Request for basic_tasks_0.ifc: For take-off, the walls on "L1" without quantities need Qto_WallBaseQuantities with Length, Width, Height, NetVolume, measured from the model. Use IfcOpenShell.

First a look at what the model holds.

```python
import ifcopenshell
import ifcopenshell.util.element
import ifcopenshell.util.unit

model = ifcopenshell.open("basic_tasks_0.ifc")
print(model.schema)
for unit_type in ("LENGTHUNIT", "AREAUNIT", "VOLUMEUNIT"):
    print(unit_type, ifcopenshell.util.unit.calculate_unit_scale(model, unit_type))
storey = next(s for s in model.by_type("IfcBuildingStorey") if s.Name == "L1")
walls = [e for e in ifcopenshell.util.element.get_decomposition(storey) if e.is_a("IfcWall")]
for e in sorted(walls, key=lambda e: e.id()):
    print(e.id(), e.is_a(), e.Name, list(ifcopenshell.util.element.get_psets(e, qtos_only=True)), sep=" | ")
```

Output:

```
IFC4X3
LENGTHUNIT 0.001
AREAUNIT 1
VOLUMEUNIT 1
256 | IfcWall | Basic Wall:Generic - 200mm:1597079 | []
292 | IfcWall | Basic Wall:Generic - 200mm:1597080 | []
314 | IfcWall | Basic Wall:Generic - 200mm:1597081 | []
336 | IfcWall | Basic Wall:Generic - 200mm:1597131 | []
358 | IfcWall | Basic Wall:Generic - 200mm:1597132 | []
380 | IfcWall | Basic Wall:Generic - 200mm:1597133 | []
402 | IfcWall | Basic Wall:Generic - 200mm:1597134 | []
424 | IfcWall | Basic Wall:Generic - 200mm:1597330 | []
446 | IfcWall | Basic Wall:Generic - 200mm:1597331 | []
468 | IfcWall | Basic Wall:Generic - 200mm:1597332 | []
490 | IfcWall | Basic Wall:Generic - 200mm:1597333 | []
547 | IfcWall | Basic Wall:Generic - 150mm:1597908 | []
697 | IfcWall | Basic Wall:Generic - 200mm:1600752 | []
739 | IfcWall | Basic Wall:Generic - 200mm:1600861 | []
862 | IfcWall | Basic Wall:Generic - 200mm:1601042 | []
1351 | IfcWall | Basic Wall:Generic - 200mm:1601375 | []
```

```python
import ifcopenshell
import ifcopenshell.api.pset
import ifcopenshell.geom
import ifcopenshell.util.element
import ifcopenshell.util.shape
import ifcopenshell.util.unit

model = ifcopenshell.open("basic_tasks_0.ifc")
unit_scale = ifcopenshell.util.unit.calculate_unit_scale(model)
volume_scale = ifcopenshell.util.unit.calculate_unit_scale(model, "VOLUMEUNIT")
settings = ifcopenshell.geom.settings()

storey = next(s for s in model.by_type("IfcBuildingStorey") if s.Name == "L1")
walls = [e for e in ifcopenshell.util.element.get_decomposition(storey) if e.is_a("IfcWall")]

for e in sorted(walls, key=lambda e: e.id()):
    if ifcopenshell.util.element.get_psets(e, qtos_only=True, should_inherit=False):
        continue
    # Geometry comes back in metres, in the element's own axes.
    shape = ifcopenshell.geom.create_shape(settings, e)
    values = {
        "Length": ifcopenshell.util.shape.get_x(shape.geometry) / unit_scale,
        "Width": ifcopenshell.util.shape.get_y(shape.geometry) / unit_scale,
        "Height": ifcopenshell.util.shape.get_z(shape.geometry) / unit_scale,
        "NetVolume": ifcopenshell.util.shape.get_volume(shape.geometry) / volume_scale,
    }
    qto = ifcopenshell.api.pset.add_qto(model, product=e, name="Qto_WallBaseQuantities")
    ifcopenshell.api.pset.edit_qto(model, qto=qto, properties=values)
    print(e.id(), {k: round(v, 3) for k, v in values.items()})

model.write("basic_tasks_0_v2.ifc")
```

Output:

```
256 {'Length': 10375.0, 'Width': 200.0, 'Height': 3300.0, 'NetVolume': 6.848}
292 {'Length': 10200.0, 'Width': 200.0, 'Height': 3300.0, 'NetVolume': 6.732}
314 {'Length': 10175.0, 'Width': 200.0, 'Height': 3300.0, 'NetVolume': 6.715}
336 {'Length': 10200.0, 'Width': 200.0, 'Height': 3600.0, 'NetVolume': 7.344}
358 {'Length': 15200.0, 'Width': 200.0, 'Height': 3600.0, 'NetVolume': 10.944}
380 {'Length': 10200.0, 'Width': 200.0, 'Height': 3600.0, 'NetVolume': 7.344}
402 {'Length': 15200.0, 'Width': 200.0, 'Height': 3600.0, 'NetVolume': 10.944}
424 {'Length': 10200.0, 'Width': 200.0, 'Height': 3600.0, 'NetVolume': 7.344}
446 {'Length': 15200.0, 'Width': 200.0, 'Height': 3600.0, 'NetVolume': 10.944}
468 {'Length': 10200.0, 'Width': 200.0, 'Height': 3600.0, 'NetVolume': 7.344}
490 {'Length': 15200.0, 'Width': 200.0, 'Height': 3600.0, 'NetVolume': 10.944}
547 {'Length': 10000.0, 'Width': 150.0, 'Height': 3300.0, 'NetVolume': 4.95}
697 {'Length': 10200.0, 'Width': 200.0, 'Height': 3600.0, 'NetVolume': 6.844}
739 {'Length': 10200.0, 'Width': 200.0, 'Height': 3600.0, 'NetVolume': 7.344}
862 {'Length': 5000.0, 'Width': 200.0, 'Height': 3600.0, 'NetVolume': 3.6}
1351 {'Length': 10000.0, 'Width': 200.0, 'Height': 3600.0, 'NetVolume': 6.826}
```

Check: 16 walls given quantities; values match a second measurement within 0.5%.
